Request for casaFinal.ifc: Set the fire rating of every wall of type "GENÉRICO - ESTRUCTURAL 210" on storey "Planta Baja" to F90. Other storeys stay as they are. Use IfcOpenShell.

First a look at what the model holds.

```python
import ifcopenshell
import ifcopenshell.util.element

model = ifcopenshell.open("casaFinal.ifc")
print(model.schema)
storey = next(s for s in model.by_type("IfcBuildingStorey") if s.Name == "Planta Baja")
walls = [e for e in ifcopenshell.util.element.get_decomposition(storey) if e.is_a("IfcWall")]
seen = {}
for e in walls:
    element_type = ifcopenshell.util.element.get_type(e)
    key = (element_type.Name if element_type != e and element_type else None, ifcopenshell.util.element.get_pset(e, "Pset_WallCommon", "FireRating"))
    seen[key] = seen.get(key, 0) + 1
for (name, value), count in sorted(seen.items(), key=str):
    print(count, "x", name, "|", value)
```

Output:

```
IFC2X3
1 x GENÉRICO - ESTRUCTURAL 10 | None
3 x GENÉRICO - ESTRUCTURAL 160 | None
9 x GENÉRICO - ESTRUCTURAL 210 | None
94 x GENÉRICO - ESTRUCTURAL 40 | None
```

```python
import ifcopenshell
import ifcopenshell.api.pset
import ifcopenshell.util.element

model = ifcopenshell.open("casaFinal.ifc")

storey = next(s for s in model.by_type("IfcBuildingStorey") if s.Name == "Planta Baja")
walls = [e for e in ifcopenshell.util.element.get_decomposition(storey) if e.is_a("IfcWall")]

count = 0
for e in walls:
    element_type = ifcopenshell.util.element.get_type(e)
    if element_type in (None, e) or element_type.Name != "GENÉRICO - ESTRUCTURAL 210":
        continue
    # add_pset returns the element's existing set when there is one.
    pset = ifcopenshell.api.pset.add_pset(model, product=e, name="Pset_WallCommon")
    ifcopenshell.api.pset.edit_pset(model, pset=pset, properties={"FireRating": "F90"})
    count += 1

print(count, "walls updated")

model.write("casaFinal_updated.ifc")
```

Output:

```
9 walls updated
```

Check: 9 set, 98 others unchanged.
